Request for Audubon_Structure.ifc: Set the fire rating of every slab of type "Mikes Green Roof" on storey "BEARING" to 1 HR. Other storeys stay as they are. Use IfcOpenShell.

First a look at what the model holds.

```python
import ifcopenshell
import ifcopenshell.util.element

model = ifcopenshell.open("Audubon_Structure.ifc")
print(model.schema)
storey = next(s for s in model.by_type("IfcBuildingStorey") if s.Name == "BEARING")
slabs = [e for e in ifcopenshell.util.element.get_decomposition(storey) if e.is_a("IfcSlab")]
seen = {}
for e in slabs:
    element_type = ifcopenshell.util.element.get_type(e)
    key = (element_type.Name if element_type != e and element_type else None, ifcopenshell.util.element.get_pset(e, "Pset_SlabCommon", "FireRating"))
    seen[key] = seen.get(key, 0) + 1
for (name, value), count in sorted(seen.items(), key=str):
    print(count, "x", name, "|", value)
```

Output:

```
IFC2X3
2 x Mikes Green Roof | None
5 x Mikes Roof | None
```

```python
import ifcopenshell
import ifcopenshell.api.pset
import ifcopenshell.util.element

model = ifcopenshell.open("Audubon_Structure.ifc")

storey = next(s for s in model.by_type("IfcBuildingStorey") if s.Name == "BEARING")
slabs = [e for e in ifcopenshell.util.element.get_decomposition(storey) if e.is_a("IfcSlab")]

count = 0
for e in slabs:
    element_type = ifcopenshell.util.element.get_type(e)
    if element_type in (None, e) or element_type.Name != "Mikes Green Roof":
        continue
    # add_pset returns the element's existing set when there is one.
    pset = ifcopenshell.api.pset.add_pset(model, product=e, name="Pset_SlabCommon")
    ifcopenshell.api.pset.edit_pset(model, pset=pset, properties={"FireRating": "1 HR"})
    count += 1

print(count, "slabs updated")

model.write("Audubon_Structure_edited.ifc")
```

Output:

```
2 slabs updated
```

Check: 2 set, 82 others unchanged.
